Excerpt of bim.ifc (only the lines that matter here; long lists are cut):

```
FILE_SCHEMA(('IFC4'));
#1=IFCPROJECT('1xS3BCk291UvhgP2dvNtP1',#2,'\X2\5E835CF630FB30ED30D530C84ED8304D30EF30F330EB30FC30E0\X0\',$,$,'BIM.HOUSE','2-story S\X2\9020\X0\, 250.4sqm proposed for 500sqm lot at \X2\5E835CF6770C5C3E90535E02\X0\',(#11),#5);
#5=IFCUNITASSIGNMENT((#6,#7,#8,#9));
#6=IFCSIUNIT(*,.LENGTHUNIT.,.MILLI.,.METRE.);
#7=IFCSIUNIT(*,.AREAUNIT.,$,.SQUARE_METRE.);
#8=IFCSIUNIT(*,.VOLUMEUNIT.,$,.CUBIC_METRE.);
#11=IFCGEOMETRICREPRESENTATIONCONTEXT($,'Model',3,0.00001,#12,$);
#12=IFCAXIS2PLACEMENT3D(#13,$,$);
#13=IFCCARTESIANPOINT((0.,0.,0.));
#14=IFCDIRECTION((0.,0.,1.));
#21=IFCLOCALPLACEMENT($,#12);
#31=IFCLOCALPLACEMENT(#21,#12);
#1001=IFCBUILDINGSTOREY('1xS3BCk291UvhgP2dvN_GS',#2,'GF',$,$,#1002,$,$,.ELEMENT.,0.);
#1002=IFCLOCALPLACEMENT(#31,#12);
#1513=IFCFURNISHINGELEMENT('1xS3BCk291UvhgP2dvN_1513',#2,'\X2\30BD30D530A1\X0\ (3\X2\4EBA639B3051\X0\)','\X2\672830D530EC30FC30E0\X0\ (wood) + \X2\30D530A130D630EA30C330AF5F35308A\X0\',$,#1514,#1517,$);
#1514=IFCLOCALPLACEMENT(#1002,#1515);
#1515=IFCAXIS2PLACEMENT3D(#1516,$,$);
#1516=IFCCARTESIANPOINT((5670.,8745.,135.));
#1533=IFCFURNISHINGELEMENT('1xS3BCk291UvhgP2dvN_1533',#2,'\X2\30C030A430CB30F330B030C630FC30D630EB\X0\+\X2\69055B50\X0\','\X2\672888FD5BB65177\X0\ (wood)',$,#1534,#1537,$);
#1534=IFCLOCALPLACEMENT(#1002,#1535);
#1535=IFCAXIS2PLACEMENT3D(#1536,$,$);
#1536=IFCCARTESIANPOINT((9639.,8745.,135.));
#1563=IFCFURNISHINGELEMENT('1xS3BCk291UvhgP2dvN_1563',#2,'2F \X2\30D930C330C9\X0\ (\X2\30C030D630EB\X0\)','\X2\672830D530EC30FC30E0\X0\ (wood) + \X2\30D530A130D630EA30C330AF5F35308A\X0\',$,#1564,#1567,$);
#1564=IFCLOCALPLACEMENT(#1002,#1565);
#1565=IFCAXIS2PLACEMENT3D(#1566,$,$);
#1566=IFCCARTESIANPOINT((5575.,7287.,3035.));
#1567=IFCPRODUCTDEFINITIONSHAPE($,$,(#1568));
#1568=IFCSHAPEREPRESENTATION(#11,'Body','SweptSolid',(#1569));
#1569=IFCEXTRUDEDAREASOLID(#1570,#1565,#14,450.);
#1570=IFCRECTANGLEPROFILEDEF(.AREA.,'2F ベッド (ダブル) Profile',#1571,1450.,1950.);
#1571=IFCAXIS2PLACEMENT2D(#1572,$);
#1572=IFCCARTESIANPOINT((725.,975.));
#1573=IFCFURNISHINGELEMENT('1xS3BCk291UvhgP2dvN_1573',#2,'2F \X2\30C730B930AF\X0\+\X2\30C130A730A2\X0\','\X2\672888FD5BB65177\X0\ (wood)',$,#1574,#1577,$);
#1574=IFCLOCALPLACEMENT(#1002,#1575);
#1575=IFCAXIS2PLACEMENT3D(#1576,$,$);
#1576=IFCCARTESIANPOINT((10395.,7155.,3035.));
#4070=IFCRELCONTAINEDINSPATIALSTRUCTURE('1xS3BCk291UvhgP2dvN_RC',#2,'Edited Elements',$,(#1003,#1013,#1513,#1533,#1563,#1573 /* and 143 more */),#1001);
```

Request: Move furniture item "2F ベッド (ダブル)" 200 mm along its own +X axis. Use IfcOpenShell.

```python
import ifcopenshell
import ifcopenshell.api.geometry
import ifcopenshell.util.placement

model = ifcopenshell.open("bim.ifc")

item = model.by_id(1563)
matrix = ifcopenshell.util.placement.get_local_placement(item.ObjectPlacement)
matrix[:3, 3] += matrix[:3, 0] * 200.0
ifcopenshell.api.geometry.edit_object_placement(model, product=item, matrix=matrix, is_si=False)

print(ifcopenshell.util.placement.get_local_placement(item.ObjectPlacement).round(3) + 0.0)

model.write("bim-out.ifc")
```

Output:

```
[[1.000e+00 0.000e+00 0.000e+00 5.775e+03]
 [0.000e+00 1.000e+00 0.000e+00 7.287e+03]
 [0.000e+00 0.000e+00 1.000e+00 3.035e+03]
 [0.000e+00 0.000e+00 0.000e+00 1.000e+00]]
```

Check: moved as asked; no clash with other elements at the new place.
